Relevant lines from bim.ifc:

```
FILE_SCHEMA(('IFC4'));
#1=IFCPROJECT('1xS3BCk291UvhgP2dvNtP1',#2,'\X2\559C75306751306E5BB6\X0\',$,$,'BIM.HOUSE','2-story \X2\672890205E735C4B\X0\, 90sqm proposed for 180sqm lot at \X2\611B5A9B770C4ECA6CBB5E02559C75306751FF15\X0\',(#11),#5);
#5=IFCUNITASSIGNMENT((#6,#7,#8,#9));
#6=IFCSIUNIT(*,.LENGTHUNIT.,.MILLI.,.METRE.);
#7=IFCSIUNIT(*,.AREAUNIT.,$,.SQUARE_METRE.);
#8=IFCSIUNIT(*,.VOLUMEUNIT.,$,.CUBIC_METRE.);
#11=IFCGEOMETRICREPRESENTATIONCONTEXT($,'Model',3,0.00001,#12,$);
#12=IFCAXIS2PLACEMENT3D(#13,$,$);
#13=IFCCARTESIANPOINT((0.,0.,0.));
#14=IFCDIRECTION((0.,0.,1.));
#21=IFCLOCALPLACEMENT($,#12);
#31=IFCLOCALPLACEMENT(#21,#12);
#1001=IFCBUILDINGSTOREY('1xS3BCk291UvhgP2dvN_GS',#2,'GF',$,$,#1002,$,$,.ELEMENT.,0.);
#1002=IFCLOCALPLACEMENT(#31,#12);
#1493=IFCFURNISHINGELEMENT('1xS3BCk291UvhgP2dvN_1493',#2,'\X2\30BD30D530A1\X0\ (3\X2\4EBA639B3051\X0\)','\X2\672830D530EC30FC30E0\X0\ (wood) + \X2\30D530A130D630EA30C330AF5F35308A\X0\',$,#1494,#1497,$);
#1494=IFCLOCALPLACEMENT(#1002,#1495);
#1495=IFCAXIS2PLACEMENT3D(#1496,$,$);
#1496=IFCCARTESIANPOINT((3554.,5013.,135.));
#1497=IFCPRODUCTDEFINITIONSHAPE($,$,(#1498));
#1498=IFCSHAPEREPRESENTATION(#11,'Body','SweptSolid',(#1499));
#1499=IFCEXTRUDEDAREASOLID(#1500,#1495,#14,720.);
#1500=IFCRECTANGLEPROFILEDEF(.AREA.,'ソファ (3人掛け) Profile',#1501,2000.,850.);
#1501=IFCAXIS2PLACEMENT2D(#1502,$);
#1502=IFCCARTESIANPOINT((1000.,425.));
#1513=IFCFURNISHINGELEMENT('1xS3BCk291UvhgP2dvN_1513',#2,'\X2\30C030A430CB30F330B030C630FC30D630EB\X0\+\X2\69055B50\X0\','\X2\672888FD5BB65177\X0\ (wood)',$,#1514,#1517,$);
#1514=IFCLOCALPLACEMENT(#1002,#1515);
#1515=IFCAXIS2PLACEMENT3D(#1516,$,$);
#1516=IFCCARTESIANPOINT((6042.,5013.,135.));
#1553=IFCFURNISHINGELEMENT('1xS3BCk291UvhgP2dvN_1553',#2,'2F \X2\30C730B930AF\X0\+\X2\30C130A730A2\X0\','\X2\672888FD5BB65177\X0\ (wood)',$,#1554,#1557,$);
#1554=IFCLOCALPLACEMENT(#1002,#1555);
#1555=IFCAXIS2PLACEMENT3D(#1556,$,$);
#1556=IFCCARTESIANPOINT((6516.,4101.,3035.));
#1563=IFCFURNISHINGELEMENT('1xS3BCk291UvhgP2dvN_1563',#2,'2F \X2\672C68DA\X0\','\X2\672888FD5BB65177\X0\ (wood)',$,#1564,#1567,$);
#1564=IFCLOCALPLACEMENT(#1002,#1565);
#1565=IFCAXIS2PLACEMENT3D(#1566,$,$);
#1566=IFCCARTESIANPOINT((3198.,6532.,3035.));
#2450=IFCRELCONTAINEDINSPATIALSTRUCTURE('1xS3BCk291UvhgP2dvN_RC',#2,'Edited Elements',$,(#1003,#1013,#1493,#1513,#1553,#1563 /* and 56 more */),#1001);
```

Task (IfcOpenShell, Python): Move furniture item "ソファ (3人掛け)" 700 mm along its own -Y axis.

```python
import ifcopenshell
import ifcopenshell.api.geometry
import ifcopenshell.util.placement

model = ifcopenshell.open("bim.ifc")

item = model.by_id(1493)
matrix = ifcopenshell.util.placement.get_local_placement(item.ObjectPlacement)
matrix[:3, 3] -= matrix[:3, 1] * 700.0
ifcopenshell.api.geometry.edit_object_placement(model, product=item, matrix=matrix, is_si=False)

print(ifcopenshell.util.placement.get_local_placement(item.ObjectPlacement).round(3) + 0.0)

model.write("bim_rev.ifc")
```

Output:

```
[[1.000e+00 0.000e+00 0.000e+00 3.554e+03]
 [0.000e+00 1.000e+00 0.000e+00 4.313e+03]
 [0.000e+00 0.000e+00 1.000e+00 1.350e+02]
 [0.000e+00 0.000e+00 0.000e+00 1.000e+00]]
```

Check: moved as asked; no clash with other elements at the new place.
